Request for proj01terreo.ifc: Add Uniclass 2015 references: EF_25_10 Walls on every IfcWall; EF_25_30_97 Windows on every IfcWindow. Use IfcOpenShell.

First a look at what the model holds.

```python
import ifcopenshell

model = ifcopenshell.open("proj01terreo.ifc")
print(model.schema)
print("classifications:", [c.Name for c in model.by_type("IfcClassification")])
for ifc_class in ("IfcDoor", "IfcRoof", "IfcStair", "IfcWall", "IfcWindow"):
    print(ifc_class, len(model.by_type(ifc_class)))
```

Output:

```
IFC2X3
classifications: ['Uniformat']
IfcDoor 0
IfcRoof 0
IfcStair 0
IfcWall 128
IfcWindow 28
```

```python
import ifcopenshell
import ifcopenshell.api.classification

model = ifcopenshell.open("proj01terreo.ifc")

# IFC2X3 requires Source and Edition and has no link from the project to the system.
system = model.create_entity("IfcClassification", Source="NBS", Edition="2015", Name="Uniclass 2015")

codes = {
    "IfcWall": ("EF_25_10", "Walls"),
    "IfcWindow": ("EF_25_30_97", "Windows"),
}
for ifc_class, (code, name) in codes.items():
    products = model.by_type(ifc_class)
    ifcopenshell.api.classification.add_reference(
        model, products=products, classification=system, identification=code, name=name
    )
    print(code, len(products))

model.write("proj01terreo_updated.ifc")
```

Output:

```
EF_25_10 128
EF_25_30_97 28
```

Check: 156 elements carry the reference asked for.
